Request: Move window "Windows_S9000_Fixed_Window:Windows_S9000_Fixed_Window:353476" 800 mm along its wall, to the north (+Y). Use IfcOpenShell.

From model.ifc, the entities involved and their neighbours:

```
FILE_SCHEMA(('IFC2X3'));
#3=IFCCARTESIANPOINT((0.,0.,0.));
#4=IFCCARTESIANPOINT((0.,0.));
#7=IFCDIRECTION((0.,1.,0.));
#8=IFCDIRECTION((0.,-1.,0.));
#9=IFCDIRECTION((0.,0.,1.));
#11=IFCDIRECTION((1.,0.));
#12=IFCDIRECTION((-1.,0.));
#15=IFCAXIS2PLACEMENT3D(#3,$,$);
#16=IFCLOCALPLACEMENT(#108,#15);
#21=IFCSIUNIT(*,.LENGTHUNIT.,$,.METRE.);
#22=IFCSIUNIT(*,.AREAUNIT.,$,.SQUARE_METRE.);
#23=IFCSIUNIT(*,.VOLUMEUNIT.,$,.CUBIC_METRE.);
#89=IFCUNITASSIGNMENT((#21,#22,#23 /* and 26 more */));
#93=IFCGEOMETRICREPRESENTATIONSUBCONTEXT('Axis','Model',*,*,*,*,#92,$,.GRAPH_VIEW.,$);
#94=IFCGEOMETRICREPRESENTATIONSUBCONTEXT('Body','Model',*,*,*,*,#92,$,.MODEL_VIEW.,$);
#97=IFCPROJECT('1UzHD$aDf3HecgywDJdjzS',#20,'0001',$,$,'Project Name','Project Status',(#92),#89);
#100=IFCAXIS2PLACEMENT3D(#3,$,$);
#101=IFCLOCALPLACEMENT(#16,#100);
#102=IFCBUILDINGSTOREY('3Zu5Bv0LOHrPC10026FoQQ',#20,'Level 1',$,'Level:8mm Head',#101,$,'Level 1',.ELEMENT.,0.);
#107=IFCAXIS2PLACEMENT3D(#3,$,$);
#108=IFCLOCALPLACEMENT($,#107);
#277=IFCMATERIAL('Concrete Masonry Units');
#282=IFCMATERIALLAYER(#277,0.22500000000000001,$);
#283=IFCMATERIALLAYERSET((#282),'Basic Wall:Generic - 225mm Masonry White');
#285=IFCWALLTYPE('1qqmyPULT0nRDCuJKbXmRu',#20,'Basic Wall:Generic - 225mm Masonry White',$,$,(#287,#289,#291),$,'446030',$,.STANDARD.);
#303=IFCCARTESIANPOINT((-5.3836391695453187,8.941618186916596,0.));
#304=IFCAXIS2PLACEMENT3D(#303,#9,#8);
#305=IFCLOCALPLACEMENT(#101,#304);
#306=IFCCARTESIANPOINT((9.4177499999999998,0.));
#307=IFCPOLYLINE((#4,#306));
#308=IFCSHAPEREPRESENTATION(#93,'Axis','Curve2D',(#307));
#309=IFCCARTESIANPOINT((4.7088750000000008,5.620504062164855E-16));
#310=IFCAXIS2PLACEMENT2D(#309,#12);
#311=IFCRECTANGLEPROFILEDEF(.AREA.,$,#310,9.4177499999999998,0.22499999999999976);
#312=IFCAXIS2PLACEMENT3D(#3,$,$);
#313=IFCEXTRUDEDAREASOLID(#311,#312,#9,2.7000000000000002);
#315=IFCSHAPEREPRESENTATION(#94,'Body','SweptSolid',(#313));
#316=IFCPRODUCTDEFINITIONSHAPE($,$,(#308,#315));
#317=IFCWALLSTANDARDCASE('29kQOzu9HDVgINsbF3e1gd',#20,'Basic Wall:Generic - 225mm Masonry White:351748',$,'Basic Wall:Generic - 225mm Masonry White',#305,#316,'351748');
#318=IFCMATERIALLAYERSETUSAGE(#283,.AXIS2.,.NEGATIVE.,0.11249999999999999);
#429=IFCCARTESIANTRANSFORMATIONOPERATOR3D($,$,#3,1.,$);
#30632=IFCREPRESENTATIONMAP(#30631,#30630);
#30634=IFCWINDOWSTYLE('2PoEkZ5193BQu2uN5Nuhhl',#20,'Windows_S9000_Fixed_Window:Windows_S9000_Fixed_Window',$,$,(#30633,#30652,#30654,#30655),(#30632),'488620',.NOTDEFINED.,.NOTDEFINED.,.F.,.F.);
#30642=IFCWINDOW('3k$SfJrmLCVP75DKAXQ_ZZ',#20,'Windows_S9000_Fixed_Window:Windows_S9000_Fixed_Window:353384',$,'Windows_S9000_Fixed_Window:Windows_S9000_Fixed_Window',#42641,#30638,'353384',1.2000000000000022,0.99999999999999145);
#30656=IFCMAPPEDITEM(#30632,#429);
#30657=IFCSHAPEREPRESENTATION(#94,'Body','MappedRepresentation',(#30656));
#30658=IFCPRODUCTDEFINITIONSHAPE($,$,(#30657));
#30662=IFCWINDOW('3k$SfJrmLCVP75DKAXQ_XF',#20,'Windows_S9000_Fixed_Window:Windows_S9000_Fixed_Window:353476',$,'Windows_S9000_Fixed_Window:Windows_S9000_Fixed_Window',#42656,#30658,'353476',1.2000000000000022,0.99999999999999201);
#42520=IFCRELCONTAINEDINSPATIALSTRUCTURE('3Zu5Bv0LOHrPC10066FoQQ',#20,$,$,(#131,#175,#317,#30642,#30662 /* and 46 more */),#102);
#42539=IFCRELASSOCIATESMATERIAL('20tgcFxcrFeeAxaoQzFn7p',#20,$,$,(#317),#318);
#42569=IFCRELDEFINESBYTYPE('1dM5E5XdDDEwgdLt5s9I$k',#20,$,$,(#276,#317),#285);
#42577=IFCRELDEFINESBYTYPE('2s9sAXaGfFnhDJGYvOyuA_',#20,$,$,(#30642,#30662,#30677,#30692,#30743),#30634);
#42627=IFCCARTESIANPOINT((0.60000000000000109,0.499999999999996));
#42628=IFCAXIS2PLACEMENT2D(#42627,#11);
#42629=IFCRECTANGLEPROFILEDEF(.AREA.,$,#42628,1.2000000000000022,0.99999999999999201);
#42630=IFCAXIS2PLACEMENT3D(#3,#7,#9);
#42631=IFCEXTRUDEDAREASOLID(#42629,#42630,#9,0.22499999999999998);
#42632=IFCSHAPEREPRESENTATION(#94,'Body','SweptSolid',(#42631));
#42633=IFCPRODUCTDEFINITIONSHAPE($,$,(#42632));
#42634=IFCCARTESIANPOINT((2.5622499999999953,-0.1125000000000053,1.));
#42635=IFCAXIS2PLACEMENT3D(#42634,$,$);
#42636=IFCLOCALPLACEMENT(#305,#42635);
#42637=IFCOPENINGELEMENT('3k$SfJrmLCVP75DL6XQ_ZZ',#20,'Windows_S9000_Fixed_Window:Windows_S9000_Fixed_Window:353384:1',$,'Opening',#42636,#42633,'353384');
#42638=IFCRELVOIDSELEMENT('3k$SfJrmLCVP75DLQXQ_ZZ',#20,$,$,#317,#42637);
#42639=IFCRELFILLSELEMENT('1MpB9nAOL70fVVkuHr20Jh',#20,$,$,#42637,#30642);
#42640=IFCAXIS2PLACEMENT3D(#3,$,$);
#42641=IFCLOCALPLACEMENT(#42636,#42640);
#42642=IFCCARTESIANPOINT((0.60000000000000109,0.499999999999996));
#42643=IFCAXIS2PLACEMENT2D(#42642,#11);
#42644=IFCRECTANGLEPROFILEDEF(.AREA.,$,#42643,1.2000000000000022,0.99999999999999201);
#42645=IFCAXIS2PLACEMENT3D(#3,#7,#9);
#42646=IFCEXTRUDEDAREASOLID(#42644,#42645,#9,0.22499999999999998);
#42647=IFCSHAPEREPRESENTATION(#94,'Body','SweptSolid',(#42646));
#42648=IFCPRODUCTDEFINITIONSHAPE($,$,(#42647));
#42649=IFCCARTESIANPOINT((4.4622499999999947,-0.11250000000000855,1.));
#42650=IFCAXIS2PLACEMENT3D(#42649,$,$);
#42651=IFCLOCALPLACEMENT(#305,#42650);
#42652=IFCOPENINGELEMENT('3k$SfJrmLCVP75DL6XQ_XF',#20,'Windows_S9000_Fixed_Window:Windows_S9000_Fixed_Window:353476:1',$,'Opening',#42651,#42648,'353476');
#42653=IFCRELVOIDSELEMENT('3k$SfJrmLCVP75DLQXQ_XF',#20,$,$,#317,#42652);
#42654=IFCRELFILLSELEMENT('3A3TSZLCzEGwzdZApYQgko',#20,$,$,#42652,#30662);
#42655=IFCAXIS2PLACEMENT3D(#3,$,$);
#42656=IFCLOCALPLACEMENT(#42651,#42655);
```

```python
import ifcopenshell
import ifcopenshell.api.geometry
import ifcopenshell.util.placement

model = ifcopenshell.open("model.ifc")

window = model.by_guid("3k$SfJrmLCVP75DKAXQ_XF")
opening = window.FillsVoids[0].RelatingOpeningElement
wall = opening.VoidsElements[0].RelatingBuildingElement

wall_matrix = ifcopenshell.util.placement.get_local_placement(wall.ObjectPlacement)
shift = wall_matrix[:3, 0] * -0.8
before = ifcopenshell.util.placement.get_local_placement(window.ObjectPlacement)[:3, 3].copy()

# The window is placed relative to its opening, so it follows when the opening moves.
matrix = ifcopenshell.util.placement.get_local_placement(opening.ObjectPlacement)
matrix[:3, 3] += shift
ifcopenshell.api.geometry.edit_object_placement(
    model, product=opening, matrix=matrix, is_si=False, should_transform_children=True
)

after = ifcopenshell.util.placement.get_local_placement(window.ObjectPlacement)[:3, 3]
print("window moved by", (after - before).round(3) + 0.0)

model.write("model_updated.ifc")
```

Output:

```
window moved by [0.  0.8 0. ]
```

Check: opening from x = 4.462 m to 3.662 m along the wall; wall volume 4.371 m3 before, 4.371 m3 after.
